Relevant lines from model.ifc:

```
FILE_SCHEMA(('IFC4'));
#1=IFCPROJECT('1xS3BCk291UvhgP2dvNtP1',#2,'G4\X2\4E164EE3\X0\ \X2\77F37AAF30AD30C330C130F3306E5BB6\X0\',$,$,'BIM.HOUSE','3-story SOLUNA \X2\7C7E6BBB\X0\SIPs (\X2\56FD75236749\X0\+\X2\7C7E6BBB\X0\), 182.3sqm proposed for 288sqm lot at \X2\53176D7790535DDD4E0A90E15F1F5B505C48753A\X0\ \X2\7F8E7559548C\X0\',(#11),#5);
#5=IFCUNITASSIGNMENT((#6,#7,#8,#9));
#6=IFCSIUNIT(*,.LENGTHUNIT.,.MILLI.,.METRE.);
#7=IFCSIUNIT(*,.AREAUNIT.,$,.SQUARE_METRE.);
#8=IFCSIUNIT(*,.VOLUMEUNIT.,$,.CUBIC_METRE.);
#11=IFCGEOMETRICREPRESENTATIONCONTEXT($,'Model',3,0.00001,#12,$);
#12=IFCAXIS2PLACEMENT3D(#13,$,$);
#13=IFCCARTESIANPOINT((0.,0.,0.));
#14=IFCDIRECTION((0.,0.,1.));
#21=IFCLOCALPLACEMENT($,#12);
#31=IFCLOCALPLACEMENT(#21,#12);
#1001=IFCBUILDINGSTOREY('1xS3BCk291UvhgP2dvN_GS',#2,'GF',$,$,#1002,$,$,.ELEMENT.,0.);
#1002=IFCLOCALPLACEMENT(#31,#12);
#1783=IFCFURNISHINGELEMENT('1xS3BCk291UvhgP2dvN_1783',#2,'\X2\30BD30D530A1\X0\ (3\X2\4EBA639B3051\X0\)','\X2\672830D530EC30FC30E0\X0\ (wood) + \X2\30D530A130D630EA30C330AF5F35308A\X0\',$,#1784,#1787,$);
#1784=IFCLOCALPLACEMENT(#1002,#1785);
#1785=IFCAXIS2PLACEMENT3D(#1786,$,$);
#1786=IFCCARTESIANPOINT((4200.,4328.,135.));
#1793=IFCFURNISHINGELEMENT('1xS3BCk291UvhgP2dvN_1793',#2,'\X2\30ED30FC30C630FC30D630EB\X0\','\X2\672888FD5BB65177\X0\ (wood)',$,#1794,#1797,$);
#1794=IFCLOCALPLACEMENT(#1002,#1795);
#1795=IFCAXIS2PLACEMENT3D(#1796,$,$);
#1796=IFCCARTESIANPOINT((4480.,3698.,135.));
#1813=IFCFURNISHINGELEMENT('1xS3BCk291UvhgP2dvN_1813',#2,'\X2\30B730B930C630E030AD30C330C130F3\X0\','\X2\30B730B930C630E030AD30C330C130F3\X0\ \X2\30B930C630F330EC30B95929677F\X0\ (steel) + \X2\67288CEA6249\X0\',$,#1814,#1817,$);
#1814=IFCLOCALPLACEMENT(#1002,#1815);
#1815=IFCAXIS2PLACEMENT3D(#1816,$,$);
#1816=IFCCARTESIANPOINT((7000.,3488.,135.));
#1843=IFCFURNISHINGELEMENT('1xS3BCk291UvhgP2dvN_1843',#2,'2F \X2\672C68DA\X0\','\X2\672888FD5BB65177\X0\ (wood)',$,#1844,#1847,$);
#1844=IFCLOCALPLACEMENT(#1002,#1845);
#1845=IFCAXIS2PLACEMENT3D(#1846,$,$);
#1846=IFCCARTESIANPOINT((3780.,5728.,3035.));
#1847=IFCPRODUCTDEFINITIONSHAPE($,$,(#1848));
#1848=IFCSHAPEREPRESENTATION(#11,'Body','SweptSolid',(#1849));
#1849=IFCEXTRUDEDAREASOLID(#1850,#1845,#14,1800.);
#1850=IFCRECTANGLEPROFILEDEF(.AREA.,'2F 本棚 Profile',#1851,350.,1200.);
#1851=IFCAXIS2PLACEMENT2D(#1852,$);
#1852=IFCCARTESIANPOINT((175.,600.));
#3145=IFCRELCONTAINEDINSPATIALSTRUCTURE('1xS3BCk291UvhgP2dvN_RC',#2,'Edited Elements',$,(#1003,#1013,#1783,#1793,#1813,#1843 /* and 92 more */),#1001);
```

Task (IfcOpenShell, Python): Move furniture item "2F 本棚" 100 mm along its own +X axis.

```python
import ifcopenshell
import ifcopenshell.api.geometry
import ifcopenshell.util.placement
import ifcopenshell.util.unit

model = ifcopenshell.open("model.ifc")
unit_scale = ifcopenshell.util.unit.calculate_unit_scale(model)

item = model.by_guid("1xS3BCk291UvhgP2dvN_1843")
matrix = ifcopenshell.util.placement.get_local_placement(item.ObjectPlacement)
matrix[:3, 3] += matrix[:3, 0] * 0.1 / unit_scale
ifcopenshell.api.geometry.edit_object_placement(model, product=item, matrix=matrix, is_si=False)

print(ifcopenshell.util.placement.get_local_placement(item.ObjectPlacement).round(3) + 0.0)

model.write("model_rev.ifc")
```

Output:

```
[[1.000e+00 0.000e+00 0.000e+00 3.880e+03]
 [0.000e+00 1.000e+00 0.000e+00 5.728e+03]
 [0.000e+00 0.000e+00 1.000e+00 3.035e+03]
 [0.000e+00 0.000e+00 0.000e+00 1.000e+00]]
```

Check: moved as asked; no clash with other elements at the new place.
